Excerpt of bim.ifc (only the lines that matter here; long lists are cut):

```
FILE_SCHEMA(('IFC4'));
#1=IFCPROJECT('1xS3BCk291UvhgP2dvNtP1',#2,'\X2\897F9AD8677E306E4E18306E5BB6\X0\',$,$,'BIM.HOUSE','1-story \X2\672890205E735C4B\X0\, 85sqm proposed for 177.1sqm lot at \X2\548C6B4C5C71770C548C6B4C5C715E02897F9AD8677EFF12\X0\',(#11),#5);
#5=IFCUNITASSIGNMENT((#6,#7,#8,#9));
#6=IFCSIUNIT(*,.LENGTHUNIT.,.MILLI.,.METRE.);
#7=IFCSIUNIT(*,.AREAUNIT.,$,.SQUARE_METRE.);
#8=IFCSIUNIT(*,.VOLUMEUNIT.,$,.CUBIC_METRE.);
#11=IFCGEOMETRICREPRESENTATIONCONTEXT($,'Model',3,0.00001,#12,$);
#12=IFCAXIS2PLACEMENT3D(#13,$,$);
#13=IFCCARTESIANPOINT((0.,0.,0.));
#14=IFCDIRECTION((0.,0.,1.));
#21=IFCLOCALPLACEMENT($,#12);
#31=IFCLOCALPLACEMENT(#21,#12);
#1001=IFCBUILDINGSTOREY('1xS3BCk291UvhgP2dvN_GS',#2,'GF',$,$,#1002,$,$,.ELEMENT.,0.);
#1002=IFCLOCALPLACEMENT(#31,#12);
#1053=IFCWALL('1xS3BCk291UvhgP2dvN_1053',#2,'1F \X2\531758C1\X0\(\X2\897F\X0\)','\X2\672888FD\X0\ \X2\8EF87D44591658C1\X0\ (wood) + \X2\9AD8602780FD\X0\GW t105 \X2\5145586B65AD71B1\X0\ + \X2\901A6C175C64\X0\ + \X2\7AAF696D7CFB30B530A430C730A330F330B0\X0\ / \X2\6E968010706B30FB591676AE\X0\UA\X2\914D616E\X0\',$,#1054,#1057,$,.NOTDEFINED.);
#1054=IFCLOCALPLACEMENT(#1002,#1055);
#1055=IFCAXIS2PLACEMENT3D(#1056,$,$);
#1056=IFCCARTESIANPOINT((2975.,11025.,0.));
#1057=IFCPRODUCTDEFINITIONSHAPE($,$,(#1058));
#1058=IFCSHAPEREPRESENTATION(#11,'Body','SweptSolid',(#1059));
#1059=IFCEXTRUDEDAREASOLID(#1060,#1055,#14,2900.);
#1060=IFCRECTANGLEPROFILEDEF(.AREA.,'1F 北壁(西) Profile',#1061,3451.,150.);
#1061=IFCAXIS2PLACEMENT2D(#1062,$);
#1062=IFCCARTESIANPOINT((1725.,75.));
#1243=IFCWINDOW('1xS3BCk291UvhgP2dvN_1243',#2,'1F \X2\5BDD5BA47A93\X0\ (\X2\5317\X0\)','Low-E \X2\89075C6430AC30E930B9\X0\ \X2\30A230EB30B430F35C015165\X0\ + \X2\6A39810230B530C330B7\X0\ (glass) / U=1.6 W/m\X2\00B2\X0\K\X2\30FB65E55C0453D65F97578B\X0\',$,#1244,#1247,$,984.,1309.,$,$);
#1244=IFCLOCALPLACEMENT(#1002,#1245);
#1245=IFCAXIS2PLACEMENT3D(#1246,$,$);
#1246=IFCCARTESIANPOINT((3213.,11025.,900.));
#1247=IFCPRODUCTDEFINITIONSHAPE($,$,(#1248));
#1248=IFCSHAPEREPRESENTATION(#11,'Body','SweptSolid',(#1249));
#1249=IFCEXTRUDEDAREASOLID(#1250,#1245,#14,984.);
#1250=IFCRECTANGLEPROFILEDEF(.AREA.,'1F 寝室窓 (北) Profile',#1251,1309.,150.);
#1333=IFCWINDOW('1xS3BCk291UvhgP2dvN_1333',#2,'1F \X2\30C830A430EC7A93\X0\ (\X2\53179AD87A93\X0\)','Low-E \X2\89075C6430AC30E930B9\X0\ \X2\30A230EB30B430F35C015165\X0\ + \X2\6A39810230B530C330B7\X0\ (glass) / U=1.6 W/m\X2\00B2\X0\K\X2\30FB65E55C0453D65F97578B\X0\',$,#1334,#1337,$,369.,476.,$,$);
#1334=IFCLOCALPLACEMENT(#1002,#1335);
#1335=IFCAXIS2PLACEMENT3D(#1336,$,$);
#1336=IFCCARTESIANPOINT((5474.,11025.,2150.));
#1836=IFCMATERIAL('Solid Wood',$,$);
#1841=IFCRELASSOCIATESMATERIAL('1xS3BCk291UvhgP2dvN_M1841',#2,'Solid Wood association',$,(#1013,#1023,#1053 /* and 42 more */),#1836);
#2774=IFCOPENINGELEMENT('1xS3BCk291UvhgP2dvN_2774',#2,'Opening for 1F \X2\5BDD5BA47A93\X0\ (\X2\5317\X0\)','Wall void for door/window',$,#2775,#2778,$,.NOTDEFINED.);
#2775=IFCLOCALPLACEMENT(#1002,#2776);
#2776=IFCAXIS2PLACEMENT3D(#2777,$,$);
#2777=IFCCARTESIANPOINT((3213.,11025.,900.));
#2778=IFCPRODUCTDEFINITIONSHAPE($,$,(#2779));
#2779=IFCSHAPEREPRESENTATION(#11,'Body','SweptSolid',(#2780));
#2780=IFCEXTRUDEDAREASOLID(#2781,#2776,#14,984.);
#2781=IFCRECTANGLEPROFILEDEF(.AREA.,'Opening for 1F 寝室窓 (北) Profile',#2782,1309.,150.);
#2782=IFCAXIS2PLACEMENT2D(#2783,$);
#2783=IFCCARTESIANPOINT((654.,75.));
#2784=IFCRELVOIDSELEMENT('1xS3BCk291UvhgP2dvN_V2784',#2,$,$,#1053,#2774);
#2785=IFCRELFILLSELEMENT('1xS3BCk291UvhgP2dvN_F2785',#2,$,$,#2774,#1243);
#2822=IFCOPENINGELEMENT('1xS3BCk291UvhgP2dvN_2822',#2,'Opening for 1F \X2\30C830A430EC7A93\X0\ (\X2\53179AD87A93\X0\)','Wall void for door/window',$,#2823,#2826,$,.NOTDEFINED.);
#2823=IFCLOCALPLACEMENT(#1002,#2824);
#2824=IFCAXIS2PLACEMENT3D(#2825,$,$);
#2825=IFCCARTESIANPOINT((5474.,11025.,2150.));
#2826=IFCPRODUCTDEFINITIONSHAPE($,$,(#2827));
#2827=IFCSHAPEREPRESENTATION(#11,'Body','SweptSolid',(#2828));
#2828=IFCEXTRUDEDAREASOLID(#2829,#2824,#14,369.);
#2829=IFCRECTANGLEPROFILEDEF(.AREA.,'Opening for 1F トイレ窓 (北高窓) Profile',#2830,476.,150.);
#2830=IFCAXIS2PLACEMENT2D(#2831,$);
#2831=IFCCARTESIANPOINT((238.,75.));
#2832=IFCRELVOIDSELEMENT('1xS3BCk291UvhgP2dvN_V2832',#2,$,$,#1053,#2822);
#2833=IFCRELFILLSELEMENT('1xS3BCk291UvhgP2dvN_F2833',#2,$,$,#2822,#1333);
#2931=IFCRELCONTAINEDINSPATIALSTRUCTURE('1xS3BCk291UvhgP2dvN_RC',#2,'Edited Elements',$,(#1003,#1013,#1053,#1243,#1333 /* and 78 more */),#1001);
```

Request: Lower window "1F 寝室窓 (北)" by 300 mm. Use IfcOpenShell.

```python
import numpy as np
import ifcopenshell
import ifcopenshell.api.geometry
import ifcopenshell.util.placement
import ifcopenshell.util.unit

model = ifcopenshell.open("bim.ifc")
unit_scale = ifcopenshell.util.unit.calculate_unit_scale(model)

window = model.by_guid("1xS3BCk291UvhgP2dvN_1243")
opening = window.FillsVoids[0].RelatingOpeningElement
dz = -0.3 / unit_scale

shift = np.array([0.0, 0.0, dz])
# The window is not placed relative to its opening, so move both.
for product in (opening, window):
    matrix = ifcopenshell.util.placement.get_local_placement(product.ObjectPlacement)
    matrix[:3, 3] += shift
    ifcopenshell.api.geometry.edit_object_placement(model, product=product, matrix=matrix, is_si=False)

print(f"moved by {dz * unit_scale:+.3f} m")

model.write("bim_edited.ifc")
```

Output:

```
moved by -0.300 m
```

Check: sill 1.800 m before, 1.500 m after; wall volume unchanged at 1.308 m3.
